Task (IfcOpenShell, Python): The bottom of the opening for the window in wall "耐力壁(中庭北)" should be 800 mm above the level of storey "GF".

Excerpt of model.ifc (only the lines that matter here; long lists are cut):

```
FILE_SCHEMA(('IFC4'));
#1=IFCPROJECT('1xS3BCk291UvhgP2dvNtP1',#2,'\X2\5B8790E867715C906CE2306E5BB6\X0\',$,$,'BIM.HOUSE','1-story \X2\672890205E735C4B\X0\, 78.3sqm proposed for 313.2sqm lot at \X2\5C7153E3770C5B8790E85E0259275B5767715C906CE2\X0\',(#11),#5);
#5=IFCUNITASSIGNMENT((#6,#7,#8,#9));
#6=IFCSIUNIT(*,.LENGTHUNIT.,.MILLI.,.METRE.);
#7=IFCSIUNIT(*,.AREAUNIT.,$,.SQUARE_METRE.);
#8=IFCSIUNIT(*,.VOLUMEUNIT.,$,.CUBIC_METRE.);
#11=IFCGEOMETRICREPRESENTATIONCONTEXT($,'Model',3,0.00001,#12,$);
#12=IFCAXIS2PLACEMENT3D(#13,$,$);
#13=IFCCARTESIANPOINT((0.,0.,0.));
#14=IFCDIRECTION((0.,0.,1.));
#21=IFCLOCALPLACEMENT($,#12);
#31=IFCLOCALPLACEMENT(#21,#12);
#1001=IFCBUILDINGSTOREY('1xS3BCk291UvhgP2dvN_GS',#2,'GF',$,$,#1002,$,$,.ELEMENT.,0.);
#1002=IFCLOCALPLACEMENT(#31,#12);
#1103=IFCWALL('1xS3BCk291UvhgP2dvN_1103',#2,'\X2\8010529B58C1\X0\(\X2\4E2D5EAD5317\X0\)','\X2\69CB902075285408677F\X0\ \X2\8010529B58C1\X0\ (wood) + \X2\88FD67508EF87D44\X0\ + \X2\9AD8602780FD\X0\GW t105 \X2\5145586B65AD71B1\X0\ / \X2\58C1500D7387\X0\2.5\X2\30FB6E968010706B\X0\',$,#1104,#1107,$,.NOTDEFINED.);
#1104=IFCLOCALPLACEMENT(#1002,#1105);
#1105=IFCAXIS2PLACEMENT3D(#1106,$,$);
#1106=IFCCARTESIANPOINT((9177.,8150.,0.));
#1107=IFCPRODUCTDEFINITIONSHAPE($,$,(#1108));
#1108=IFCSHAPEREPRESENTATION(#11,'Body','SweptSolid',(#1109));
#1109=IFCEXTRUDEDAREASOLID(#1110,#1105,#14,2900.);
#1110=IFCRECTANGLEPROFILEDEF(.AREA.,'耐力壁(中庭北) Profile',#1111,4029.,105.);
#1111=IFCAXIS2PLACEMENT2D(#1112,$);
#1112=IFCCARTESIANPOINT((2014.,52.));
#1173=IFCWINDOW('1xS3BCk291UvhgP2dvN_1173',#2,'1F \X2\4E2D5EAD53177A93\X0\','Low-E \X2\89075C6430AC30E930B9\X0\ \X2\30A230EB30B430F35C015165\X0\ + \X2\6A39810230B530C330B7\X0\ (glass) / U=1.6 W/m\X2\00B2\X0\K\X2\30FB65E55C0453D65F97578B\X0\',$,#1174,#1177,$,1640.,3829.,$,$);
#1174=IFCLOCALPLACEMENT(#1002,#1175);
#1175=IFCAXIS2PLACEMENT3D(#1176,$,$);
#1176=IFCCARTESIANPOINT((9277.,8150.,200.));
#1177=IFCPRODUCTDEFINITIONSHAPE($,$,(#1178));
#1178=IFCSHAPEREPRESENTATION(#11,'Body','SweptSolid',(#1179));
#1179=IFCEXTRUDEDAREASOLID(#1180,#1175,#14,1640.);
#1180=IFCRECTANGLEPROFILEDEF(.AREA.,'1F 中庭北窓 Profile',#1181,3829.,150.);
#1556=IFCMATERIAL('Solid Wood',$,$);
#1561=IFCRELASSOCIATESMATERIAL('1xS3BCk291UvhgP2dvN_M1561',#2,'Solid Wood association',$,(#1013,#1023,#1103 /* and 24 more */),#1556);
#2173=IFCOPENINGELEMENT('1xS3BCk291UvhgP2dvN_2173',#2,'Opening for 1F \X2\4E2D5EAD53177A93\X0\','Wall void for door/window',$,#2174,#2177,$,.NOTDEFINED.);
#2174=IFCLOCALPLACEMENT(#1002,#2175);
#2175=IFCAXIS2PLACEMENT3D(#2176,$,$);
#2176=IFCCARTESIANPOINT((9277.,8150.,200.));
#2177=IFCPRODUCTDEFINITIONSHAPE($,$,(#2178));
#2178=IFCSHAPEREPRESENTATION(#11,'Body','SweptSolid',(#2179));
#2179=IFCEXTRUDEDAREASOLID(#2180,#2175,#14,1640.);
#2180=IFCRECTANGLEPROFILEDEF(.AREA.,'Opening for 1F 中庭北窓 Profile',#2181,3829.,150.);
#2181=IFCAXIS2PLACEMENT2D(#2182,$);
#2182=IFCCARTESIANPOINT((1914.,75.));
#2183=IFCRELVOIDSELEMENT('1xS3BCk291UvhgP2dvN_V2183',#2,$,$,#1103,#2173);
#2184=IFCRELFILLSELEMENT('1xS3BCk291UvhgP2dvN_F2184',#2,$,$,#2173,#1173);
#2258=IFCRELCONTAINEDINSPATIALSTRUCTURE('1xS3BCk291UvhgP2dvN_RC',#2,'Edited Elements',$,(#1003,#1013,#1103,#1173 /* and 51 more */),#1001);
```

```python
import numpy as np
import ifcopenshell
import ifcopenshell.api.geometry
import ifcopenshell.geom
import ifcopenshell.util.element
import ifcopenshell.util.placement
import ifcopenshell.util.shape
import ifcopenshell.util.unit

model = ifcopenshell.open("model.ifc")
unit_scale = ifcopenshell.util.unit.calculate_unit_scale(model)

window = model.by_guid("1xS3BCk291UvhgP2dvN_1173")
opening = window.FillsVoids[0].RelatingOpeningElement
storey = ifcopenshell.util.element.get_container(window, ifc_class="IfcBuildingStorey")
level = ifcopenshell.util.placement.get_local_placement(storey.ObjectPlacement)[2, 3]

# The opening's origin need not be at the sill, so measure its lowest point.
shape = ifcopenshell.geom.create_shape(ifcopenshell.geom.settings(), opening)
bottom = ifcopenshell.util.shape.get_shape_bottom_elevation(shape, shape.geometry) / unit_scale
dz = level + 0.8 / unit_scale - bottom

shift = np.array([0.0, 0.0, dz])
# The window is not placed relative to its opening, so move both.
for product in (opening, window):
    matrix = ifcopenshell.util.placement.get_local_placement(product.ObjectPlacement)
    matrix[:3, 3] += shift
    ifcopenshell.api.geometry.edit_object_placement(model, product=product, matrix=matrix, is_si=False)

print(f"moved by {dz * unit_scale:+.3f} m")

model.write("model_rev.ifc")
```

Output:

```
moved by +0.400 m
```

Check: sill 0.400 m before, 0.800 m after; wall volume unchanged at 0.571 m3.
